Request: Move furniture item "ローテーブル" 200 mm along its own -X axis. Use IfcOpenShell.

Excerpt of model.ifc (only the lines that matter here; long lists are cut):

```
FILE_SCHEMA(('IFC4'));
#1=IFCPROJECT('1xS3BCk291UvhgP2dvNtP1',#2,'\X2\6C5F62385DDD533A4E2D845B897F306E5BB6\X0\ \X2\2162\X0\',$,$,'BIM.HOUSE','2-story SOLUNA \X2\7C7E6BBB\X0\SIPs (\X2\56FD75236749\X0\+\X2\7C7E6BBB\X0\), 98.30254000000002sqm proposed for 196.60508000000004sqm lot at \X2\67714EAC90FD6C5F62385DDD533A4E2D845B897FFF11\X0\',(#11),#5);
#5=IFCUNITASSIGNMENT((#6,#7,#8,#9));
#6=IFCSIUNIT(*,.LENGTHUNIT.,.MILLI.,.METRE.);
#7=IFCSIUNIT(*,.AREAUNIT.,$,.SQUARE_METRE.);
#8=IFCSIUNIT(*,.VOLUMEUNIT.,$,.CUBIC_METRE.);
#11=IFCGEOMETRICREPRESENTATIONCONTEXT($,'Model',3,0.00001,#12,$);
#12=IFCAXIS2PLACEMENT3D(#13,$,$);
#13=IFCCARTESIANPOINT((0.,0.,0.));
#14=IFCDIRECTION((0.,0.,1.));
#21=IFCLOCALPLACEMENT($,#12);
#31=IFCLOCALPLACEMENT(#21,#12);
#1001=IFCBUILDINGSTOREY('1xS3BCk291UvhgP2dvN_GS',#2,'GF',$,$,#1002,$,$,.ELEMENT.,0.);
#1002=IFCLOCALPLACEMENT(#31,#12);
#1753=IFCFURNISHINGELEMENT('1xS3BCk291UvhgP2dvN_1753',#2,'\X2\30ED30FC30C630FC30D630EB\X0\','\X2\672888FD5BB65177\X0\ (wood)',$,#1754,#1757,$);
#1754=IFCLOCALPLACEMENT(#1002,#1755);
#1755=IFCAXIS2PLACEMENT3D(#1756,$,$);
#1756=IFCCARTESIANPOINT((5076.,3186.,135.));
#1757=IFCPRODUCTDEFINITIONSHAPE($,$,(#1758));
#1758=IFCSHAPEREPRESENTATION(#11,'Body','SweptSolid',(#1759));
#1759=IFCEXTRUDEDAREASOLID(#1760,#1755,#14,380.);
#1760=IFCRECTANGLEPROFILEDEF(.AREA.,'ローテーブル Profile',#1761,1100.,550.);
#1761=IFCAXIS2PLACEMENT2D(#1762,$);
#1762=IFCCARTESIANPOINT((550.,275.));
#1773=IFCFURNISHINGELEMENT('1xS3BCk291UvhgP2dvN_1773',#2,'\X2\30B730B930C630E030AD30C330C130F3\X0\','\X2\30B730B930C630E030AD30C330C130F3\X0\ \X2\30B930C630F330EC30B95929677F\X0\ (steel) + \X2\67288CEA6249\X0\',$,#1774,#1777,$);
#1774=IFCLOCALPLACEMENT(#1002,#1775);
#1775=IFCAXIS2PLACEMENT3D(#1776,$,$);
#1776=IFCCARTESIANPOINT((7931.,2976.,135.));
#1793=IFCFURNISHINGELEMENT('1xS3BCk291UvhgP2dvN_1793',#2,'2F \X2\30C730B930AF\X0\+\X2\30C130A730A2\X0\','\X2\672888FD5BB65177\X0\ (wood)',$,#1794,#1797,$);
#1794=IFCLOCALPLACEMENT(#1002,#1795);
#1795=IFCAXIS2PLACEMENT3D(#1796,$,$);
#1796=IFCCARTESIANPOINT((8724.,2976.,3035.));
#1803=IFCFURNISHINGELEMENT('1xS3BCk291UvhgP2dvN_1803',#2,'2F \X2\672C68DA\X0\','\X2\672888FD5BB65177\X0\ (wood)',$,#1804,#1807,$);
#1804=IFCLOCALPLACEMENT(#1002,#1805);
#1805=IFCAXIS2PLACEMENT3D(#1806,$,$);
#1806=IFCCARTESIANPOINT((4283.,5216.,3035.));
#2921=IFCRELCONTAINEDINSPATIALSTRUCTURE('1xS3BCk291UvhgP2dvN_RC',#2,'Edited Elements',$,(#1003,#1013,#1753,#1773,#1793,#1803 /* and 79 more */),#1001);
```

```python
import ifcopenshell
import ifcopenshell.api.geometry
import ifcopenshell.util.placement

model = ifcopenshell.open("model.ifc")

item = model.by_guid("1xS3BCk291UvhgP2dvN_1753")
matrix = ifcopenshell.util.placement.get_local_placement(item.ObjectPlacement)
matrix[:3, 3] -= matrix[:3, 0] * 200.0
ifcopenshell.api.geometry.edit_object_placement(model, product=item, matrix=matrix, is_si=False)

print(ifcopenshell.util.placement.get_local_placement(item.ObjectPlacement).round(3) + 0.0)

model.write("model_rev.ifc")
```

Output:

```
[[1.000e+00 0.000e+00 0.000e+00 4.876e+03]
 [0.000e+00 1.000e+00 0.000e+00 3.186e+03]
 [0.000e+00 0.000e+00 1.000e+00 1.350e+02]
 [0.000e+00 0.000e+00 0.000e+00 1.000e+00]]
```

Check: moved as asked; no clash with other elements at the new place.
